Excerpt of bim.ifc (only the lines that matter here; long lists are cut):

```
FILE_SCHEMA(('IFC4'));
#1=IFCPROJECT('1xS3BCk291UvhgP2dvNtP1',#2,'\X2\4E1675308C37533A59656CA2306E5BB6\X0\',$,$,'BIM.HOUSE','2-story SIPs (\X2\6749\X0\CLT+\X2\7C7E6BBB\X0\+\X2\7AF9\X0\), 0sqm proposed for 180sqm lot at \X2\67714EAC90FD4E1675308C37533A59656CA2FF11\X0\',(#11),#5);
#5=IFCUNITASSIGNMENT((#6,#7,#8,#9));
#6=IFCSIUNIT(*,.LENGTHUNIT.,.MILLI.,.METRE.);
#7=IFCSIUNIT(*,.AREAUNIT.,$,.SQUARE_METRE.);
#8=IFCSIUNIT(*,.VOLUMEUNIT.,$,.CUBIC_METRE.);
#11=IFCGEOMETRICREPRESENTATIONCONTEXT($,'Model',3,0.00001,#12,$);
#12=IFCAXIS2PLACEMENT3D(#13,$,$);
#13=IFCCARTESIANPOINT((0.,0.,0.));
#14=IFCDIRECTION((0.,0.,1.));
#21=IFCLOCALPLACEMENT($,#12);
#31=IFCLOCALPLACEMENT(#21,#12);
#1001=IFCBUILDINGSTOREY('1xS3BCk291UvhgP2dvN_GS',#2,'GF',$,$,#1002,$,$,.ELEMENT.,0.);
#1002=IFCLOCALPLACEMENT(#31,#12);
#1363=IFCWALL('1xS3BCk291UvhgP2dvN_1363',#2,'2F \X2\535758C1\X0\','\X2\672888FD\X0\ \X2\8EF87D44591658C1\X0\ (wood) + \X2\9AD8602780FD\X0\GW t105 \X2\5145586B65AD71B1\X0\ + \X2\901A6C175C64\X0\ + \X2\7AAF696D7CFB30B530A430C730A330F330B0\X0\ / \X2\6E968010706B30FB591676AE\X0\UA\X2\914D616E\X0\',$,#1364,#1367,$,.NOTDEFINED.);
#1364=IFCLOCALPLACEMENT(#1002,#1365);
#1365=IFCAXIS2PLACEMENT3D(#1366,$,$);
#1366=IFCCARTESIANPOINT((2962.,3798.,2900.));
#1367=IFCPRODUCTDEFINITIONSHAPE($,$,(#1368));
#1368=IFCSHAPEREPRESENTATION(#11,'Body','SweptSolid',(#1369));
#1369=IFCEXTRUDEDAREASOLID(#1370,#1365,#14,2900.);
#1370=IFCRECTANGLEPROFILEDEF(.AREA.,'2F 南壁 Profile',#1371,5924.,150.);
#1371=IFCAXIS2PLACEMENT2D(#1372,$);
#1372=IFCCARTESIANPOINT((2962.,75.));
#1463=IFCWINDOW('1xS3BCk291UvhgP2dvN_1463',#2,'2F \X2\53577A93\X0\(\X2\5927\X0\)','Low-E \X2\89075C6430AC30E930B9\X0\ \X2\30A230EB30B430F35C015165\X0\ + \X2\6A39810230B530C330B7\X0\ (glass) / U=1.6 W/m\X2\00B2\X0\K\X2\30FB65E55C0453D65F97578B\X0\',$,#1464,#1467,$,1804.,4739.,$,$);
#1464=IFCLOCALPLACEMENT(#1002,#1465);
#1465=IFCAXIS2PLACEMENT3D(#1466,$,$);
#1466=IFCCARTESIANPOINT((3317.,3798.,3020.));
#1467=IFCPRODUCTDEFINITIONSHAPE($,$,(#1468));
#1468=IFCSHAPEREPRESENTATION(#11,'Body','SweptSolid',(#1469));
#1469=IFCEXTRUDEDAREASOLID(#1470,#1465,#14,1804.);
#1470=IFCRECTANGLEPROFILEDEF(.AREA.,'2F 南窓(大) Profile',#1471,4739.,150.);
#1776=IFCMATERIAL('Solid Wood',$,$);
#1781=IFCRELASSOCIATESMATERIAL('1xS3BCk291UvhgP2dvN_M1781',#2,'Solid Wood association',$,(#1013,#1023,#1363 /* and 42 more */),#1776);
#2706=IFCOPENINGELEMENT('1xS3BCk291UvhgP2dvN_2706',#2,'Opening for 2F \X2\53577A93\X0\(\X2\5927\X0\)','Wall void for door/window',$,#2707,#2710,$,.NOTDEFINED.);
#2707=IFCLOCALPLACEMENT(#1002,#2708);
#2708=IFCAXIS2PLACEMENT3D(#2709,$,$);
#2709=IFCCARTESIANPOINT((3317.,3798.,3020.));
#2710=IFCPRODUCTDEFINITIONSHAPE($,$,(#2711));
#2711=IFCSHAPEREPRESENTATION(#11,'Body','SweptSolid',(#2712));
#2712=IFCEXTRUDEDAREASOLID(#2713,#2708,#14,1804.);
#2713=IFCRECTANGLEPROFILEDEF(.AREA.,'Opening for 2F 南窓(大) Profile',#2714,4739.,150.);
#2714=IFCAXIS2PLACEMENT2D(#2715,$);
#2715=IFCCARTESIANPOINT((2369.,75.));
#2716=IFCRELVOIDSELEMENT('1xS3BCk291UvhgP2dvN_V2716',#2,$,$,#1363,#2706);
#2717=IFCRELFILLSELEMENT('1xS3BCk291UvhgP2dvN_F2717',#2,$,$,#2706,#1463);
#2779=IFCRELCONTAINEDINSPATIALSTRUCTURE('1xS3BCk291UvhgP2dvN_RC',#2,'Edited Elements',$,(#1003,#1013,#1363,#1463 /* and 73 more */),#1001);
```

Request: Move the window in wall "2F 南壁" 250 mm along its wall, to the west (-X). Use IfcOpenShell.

```python
import ifcopenshell
import ifcopenshell.api.geometry
import ifcopenshell.util.placement

model = ifcopenshell.open("bim.ifc")

window = model.by_guid("1xS3BCk291UvhgP2dvN_1463")
opening = window.FillsVoids[0].RelatingOpeningElement
wall = opening.VoidsElements[0].RelatingBuildingElement

wall_matrix = ifcopenshell.util.placement.get_local_placement(wall.ObjectPlacement)
shift = wall_matrix[:3, 0] * -250.0
before = ifcopenshell.util.placement.get_local_placement(window.ObjectPlacement)[:3, 3].copy()

# The window is not placed relative to its opening, so move both.
for product in (opening, window):
    matrix = ifcopenshell.util.placement.get_local_placement(product.ObjectPlacement)
    matrix[:3, 3] += shift
    ifcopenshell.api.geometry.edit_object_placement(model, product=product, matrix=matrix, is_si=False)

after = ifcopenshell.util.placement.get_local_placement(window.ObjectPlacement)[:3, 3]
print("window moved by", (after - before).round(3) + 0.0)

model.write("bim_edited.ifc")
```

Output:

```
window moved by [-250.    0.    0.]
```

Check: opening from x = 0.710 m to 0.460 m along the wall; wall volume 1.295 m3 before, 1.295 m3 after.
